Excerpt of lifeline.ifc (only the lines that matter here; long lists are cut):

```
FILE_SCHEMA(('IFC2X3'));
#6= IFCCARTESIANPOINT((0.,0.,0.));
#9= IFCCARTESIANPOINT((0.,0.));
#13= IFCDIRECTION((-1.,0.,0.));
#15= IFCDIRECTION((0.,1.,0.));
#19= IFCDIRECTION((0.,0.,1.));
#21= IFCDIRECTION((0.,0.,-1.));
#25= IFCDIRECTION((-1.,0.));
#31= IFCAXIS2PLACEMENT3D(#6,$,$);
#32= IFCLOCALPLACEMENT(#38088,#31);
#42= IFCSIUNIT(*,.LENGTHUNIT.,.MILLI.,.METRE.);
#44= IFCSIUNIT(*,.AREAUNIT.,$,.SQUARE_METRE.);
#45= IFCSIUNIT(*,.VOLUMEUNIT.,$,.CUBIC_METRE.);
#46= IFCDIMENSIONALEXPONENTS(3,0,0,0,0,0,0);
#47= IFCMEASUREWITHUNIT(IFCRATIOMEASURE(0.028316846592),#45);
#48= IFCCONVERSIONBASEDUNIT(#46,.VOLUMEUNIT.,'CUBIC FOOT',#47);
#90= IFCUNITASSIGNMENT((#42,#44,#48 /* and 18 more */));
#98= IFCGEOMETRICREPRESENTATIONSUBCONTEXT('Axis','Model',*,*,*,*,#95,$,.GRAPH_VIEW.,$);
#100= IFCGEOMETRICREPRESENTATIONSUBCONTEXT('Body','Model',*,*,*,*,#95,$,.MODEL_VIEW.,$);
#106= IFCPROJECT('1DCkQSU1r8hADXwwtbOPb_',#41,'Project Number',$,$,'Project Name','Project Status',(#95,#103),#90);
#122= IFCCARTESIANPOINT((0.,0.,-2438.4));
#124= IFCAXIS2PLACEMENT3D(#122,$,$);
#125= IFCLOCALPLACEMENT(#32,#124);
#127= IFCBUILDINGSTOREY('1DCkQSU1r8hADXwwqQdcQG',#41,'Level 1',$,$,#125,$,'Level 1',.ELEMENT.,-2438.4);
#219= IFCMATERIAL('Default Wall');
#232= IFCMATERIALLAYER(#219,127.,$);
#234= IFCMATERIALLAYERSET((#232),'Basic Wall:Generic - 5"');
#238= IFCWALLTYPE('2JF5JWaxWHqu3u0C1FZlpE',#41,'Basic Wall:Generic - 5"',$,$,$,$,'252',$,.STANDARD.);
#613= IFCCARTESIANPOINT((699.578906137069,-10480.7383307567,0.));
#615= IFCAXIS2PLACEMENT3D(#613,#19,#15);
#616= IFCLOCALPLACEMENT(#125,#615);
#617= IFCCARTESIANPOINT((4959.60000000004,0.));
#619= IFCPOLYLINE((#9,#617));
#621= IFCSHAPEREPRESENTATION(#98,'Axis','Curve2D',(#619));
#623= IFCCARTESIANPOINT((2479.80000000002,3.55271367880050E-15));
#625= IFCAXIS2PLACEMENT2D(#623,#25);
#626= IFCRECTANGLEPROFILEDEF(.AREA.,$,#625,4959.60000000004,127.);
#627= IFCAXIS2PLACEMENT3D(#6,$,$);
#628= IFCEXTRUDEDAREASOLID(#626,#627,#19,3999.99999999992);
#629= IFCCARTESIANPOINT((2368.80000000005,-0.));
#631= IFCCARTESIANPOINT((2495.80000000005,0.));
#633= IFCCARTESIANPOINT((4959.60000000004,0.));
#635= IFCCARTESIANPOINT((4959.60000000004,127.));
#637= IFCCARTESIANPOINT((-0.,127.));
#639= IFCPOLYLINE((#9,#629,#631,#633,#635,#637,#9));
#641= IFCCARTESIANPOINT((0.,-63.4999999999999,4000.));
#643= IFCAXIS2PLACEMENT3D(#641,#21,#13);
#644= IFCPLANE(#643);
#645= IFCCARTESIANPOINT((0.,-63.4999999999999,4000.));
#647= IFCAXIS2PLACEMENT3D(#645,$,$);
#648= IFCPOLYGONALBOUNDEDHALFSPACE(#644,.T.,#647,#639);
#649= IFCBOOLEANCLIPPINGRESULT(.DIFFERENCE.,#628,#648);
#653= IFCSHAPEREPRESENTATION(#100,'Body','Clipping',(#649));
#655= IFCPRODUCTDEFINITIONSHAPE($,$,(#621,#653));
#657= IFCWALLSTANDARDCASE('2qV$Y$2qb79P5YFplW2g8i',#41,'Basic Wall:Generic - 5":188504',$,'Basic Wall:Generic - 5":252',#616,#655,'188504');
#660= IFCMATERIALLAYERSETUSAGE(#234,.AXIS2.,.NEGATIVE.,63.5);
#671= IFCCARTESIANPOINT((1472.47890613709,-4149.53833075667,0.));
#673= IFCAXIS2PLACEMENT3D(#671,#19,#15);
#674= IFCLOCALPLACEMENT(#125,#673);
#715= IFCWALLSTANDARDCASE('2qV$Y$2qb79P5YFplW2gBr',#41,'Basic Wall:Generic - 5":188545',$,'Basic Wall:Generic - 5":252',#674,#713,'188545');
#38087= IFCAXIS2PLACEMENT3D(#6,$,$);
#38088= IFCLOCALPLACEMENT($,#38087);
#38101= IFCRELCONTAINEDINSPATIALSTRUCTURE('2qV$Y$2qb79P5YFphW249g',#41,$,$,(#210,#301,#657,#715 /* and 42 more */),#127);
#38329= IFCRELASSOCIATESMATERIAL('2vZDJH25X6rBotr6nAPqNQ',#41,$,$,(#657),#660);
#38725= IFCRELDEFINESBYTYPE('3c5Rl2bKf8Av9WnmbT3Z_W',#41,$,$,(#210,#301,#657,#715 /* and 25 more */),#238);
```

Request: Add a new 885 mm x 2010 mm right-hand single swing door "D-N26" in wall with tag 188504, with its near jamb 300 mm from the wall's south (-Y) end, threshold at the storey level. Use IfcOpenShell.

```python
import numpy as np
import ifcopenshell
import ifcopenshell.api.feature
import ifcopenshell.api.geometry
import ifcopenshell.api.root
import ifcopenshell.api.spatial
import ifcopenshell.api.type
import ifcopenshell.geom
import ifcopenshell.util.element
import ifcopenshell.util.placement
import ifcopenshell.util.representation
import ifcopenshell.util.shape
import ifcopenshell.util.unit

model = ifcopenshell.open("lifeline.ifc")
unit_scale = ifcopenshell.util.unit.calculate_unit_scale(model)
settings = ifcopenshell.geom.settings()


def volume(element):
    """Net volume in cubic metres, openings subtracted."""
    shape = ifcopenshell.geom.create_shape(settings, element)
    return ifcopenshell.util.shape.get_volume(shape.geometry)


wall = model.by_guid("2qV$Y$2qb79P5YFplW2g8i")
storey = ifcopenshell.util.element.get_container(wall, ifc_class="IfcBuildingStorey")
context = ifcopenshell.util.representation.get_context(model, "Model", "Body", "MODEL_VIEW")
before = volume(wall)

width, height, from_end, sill = 0.885, 2.01, 0.3, 0.0  # metres

# The wall runs along its own X axis, and the end named is its -X end.
wall_shape = ifcopenshell.geom.create_shape(settings, wall)
x, y, z = ifcopenshell.util.shape.get_vertices(wall_shape.geometry).T
start = x.min() + from_end
face, thickness = float(y.min()), float(y.max() - y.min())
wall_matrix = ifcopenshell.util.placement.get_local_placement(wall.ObjectPlacement)
level = ifcopenshell.util.placement.get_local_placement(storey.ObjectPlacement)[2, 3]


def in_wall(x, y):
    """Placement at x, y metres in the wall's axes, at sill height."""
    matrix = wall_matrix.copy()
    matrix[:, 3] = wall_matrix @ np.array([x / unit_scale, y / unit_scale, 0.0, 1.0])
    matrix[2, 3] = level + sill / unit_scale
    return matrix


# Opening: a box that overshoots both wall faces by 50 mm.
opening = ifcopenshell.api.root.create_entity(model, ifc_class="IfcOpeningElement")
box = ifcopenshell.api.geometry.add_wall_representation(
    model, context=context, length=width, height=height, thickness=thickness + 0.1
)
ifcopenshell.api.geometry.assign_representation(model, product=opening, representation=box)
ifcopenshell.api.geometry.edit_object_placement(model, product=opening, matrix=in_wall(start, face - 0.05), is_si=False)
ifcopenshell.api.feature.add_feature(model, feature=opening, element=wall)

door = ifcopenshell.api.root.create_entity(model, ifc_class="IfcDoor", name="D-N26")
door.OverallWidth, door.OverallHeight = width / unit_scale, height / unit_scale
body = ifcopenshell.api.geometry.add_door_representation(
    model,
    context=context,
    overall_width=door.OverallWidth,
    overall_height=door.OverallHeight,
    operation_type="SINGLE_SWING_RIGHT",
    lining_properties={"LiningDepth": thickness / unit_scale, "ThresholdDepth": thickness / unit_scale},
)
ifcopenshell.api.geometry.assign_representation(model, product=door, representation=body)
ifcopenshell.api.spatial.assign_container(model, products=[door], relating_structure=storey)
fills = ifcopenshell.api.feature.add_filling(model, opening=opening, element=door)
fills.OwnerHistory = door.OwnerHistory  # required in IFC2X3

# IFC2X3 keeps the operation on the door style.
style = ifcopenshell.api.root.create_entity(model, ifc_class="IfcDoorStyle", name="D-N26")
style.OperationType, style.ConstructionType = "SINGLE_SWING_RIGHT", "NOTDEFINED"
style.ParameterTakesPrecedence = style.Sizeable = False
ifcopenshell.api.type.assign_type(model, related_objects=[door], relating_type=style)

# The lining spans the wall, so the door starts at the wall face.
ifcopenshell.api.geometry.edit_object_placement(model, product=door, matrix=in_wall(start, face), is_si=False)

after = volume(wall)

print(f"wall volume {before:.3f} -> {after:.3f} m3")

model.write("lifeline_updated.ifc")
```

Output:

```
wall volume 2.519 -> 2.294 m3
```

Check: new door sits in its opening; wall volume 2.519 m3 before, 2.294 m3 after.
